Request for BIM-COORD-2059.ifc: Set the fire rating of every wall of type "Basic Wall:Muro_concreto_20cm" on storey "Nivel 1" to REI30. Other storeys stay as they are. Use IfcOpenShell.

First a look at what the model holds.

```python
import ifcopenshell
import ifcopenshell.util.element

model = ifcopenshell.open("BIM-COORD-2059.ifc")
print(model.schema)
storey = next(s for s in model.by_type("IfcBuildingStorey") if s.Name == "Nivel 1")
walls = [e for e in ifcopenshell.util.element.get_decomposition(storey) if e.is_a("IfcWall")]
seen = {}
for e in walls:
    element_type = ifcopenshell.util.element.get_type(e)
    key = (element_type.Name if element_type != e and element_type else None, ifcopenshell.util.element.get_pset(e, "Pset_WallCommon", "FireRating"))
    seen[key] = seen.get(key, 0) + 1
for (name, value), count in sorted(seen.items(), key=str):
    print(count, "x", name, "|", value)
```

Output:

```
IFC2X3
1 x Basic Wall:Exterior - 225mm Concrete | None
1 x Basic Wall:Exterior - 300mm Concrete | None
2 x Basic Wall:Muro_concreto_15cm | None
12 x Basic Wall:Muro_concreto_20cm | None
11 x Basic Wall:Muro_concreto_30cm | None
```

```python
import ifcopenshell
import ifcopenshell.api.pset
import ifcopenshell.util.element

model = ifcopenshell.open("BIM-COORD-2059.ifc")

storey = next(s for s in model.by_type("IfcBuildingStorey") if s.Name == "Nivel 1")
walls = [e for e in ifcopenshell.util.element.get_decomposition(storey) if e.is_a("IfcWall")]

count = 0
for e in walls:
    element_type = ifcopenshell.util.element.get_type(e)
    if element_type in (None, e) or element_type.Name != "Basic Wall:Muro_concreto_20cm":
        continue
    # add_pset returns the element's existing set when there is one.
    pset = ifcopenshell.api.pset.add_pset(model, product=e, name="Pset_WallCommon")
    ifcopenshell.api.pset.edit_pset(model, pset=pset, properties={"FireRating": "REI30"})
    count += 1

print(count, "walls updated")

model.write("BIM-COORD-2059_v2.ifc")
```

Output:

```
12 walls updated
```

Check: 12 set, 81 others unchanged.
